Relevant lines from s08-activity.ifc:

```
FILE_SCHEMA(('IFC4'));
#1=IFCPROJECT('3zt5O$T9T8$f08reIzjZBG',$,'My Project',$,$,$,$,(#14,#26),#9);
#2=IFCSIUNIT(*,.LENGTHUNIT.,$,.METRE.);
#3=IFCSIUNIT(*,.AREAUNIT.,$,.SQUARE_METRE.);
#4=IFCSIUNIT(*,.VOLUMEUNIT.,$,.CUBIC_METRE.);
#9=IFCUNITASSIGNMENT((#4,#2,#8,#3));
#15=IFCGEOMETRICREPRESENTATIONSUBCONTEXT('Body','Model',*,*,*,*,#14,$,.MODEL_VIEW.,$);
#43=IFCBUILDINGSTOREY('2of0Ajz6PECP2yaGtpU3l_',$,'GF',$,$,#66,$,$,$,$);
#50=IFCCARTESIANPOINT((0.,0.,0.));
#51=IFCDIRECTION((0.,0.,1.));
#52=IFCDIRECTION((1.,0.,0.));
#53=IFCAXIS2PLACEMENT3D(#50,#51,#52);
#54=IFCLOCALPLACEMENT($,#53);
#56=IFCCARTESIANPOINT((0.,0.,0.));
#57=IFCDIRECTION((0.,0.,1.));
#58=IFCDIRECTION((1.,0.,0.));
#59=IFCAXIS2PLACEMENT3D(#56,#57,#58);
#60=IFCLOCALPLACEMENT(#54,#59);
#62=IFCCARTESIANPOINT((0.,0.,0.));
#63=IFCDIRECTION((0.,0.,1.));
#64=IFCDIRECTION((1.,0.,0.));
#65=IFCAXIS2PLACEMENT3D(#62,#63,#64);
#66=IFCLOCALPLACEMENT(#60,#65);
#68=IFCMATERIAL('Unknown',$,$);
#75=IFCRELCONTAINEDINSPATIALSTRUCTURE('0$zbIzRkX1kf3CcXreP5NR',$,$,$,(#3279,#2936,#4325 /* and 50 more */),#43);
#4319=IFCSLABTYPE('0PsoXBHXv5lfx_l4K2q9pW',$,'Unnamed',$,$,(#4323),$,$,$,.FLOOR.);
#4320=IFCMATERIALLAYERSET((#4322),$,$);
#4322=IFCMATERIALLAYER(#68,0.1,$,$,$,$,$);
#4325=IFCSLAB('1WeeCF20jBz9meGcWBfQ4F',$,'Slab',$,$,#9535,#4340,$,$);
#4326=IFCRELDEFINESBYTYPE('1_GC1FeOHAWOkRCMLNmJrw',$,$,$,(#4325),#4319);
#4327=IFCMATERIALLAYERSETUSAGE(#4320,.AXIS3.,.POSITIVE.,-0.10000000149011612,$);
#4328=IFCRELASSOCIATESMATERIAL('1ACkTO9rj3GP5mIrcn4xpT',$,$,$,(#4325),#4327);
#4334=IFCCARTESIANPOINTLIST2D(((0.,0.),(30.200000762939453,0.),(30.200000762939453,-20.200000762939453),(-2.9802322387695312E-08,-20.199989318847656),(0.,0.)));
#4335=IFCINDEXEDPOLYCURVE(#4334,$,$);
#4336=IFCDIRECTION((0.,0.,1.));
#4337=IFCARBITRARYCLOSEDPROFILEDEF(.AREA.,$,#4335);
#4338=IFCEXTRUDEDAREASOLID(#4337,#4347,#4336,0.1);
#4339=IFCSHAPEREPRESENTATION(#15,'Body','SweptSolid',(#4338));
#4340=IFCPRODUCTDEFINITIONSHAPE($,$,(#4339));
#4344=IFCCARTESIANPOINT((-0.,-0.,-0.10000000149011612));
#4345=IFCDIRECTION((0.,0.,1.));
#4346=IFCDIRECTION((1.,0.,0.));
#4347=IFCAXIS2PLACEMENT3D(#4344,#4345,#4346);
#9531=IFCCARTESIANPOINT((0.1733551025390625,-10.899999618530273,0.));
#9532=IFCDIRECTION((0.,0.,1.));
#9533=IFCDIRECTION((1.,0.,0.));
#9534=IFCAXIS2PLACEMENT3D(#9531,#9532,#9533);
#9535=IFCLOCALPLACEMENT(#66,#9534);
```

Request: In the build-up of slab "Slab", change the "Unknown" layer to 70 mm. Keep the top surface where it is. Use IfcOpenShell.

```python
import ifcopenshell
import ifcopenshell.util.element
import ifcopenshell.util.representation
import ifcopenshell.util.unit

model = ifcopenshell.open("s08-activity.ifc")
unit_scale = ifcopenshell.util.unit.calculate_unit_scale(model)

layer_set = model.by_id(4320)
layer = next(l for l in layer_set.MaterialLayers if l.Material and l.Material.Name == "Unknown")
change = 0.07 / unit_scale - layer.LayerThickness
layer.LayerThickness += change

# Geometry does not follow the layer set by itself.
slabs = [e for e in ifcopenshell.util.element.get_elements_by_material(model, layer_set) if e.is_a("IfcSlab")]
for slab in sorted(slabs, key=lambda e: e.id()):
    body = ifcopenshell.util.representation.get_representation(slab, "Model", "Body")
    solid = body.Items[0]
    old_depth = solid.Depth
    solid.Depth += change
    # Extruded upwards: lower the start of the extrusion so the top stays.
    x, y, z = solid.Position.Location.Coordinates
    solid.Position.Location = model.createIfcCartesianPoint((x, y, z - change))
    print(slab.id(), f"{old_depth:g} -> {solid.Depth:g}")

# The layers are counted up from the underside, which has moved.
for usage in {ifcopenshell.util.element.get_material(slab) for slab in slabs}:
    usage.OffsetFromReferenceLine -= change

model.write("s08-activity_updated.ifc")
```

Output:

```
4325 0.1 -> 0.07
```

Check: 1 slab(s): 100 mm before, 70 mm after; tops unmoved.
